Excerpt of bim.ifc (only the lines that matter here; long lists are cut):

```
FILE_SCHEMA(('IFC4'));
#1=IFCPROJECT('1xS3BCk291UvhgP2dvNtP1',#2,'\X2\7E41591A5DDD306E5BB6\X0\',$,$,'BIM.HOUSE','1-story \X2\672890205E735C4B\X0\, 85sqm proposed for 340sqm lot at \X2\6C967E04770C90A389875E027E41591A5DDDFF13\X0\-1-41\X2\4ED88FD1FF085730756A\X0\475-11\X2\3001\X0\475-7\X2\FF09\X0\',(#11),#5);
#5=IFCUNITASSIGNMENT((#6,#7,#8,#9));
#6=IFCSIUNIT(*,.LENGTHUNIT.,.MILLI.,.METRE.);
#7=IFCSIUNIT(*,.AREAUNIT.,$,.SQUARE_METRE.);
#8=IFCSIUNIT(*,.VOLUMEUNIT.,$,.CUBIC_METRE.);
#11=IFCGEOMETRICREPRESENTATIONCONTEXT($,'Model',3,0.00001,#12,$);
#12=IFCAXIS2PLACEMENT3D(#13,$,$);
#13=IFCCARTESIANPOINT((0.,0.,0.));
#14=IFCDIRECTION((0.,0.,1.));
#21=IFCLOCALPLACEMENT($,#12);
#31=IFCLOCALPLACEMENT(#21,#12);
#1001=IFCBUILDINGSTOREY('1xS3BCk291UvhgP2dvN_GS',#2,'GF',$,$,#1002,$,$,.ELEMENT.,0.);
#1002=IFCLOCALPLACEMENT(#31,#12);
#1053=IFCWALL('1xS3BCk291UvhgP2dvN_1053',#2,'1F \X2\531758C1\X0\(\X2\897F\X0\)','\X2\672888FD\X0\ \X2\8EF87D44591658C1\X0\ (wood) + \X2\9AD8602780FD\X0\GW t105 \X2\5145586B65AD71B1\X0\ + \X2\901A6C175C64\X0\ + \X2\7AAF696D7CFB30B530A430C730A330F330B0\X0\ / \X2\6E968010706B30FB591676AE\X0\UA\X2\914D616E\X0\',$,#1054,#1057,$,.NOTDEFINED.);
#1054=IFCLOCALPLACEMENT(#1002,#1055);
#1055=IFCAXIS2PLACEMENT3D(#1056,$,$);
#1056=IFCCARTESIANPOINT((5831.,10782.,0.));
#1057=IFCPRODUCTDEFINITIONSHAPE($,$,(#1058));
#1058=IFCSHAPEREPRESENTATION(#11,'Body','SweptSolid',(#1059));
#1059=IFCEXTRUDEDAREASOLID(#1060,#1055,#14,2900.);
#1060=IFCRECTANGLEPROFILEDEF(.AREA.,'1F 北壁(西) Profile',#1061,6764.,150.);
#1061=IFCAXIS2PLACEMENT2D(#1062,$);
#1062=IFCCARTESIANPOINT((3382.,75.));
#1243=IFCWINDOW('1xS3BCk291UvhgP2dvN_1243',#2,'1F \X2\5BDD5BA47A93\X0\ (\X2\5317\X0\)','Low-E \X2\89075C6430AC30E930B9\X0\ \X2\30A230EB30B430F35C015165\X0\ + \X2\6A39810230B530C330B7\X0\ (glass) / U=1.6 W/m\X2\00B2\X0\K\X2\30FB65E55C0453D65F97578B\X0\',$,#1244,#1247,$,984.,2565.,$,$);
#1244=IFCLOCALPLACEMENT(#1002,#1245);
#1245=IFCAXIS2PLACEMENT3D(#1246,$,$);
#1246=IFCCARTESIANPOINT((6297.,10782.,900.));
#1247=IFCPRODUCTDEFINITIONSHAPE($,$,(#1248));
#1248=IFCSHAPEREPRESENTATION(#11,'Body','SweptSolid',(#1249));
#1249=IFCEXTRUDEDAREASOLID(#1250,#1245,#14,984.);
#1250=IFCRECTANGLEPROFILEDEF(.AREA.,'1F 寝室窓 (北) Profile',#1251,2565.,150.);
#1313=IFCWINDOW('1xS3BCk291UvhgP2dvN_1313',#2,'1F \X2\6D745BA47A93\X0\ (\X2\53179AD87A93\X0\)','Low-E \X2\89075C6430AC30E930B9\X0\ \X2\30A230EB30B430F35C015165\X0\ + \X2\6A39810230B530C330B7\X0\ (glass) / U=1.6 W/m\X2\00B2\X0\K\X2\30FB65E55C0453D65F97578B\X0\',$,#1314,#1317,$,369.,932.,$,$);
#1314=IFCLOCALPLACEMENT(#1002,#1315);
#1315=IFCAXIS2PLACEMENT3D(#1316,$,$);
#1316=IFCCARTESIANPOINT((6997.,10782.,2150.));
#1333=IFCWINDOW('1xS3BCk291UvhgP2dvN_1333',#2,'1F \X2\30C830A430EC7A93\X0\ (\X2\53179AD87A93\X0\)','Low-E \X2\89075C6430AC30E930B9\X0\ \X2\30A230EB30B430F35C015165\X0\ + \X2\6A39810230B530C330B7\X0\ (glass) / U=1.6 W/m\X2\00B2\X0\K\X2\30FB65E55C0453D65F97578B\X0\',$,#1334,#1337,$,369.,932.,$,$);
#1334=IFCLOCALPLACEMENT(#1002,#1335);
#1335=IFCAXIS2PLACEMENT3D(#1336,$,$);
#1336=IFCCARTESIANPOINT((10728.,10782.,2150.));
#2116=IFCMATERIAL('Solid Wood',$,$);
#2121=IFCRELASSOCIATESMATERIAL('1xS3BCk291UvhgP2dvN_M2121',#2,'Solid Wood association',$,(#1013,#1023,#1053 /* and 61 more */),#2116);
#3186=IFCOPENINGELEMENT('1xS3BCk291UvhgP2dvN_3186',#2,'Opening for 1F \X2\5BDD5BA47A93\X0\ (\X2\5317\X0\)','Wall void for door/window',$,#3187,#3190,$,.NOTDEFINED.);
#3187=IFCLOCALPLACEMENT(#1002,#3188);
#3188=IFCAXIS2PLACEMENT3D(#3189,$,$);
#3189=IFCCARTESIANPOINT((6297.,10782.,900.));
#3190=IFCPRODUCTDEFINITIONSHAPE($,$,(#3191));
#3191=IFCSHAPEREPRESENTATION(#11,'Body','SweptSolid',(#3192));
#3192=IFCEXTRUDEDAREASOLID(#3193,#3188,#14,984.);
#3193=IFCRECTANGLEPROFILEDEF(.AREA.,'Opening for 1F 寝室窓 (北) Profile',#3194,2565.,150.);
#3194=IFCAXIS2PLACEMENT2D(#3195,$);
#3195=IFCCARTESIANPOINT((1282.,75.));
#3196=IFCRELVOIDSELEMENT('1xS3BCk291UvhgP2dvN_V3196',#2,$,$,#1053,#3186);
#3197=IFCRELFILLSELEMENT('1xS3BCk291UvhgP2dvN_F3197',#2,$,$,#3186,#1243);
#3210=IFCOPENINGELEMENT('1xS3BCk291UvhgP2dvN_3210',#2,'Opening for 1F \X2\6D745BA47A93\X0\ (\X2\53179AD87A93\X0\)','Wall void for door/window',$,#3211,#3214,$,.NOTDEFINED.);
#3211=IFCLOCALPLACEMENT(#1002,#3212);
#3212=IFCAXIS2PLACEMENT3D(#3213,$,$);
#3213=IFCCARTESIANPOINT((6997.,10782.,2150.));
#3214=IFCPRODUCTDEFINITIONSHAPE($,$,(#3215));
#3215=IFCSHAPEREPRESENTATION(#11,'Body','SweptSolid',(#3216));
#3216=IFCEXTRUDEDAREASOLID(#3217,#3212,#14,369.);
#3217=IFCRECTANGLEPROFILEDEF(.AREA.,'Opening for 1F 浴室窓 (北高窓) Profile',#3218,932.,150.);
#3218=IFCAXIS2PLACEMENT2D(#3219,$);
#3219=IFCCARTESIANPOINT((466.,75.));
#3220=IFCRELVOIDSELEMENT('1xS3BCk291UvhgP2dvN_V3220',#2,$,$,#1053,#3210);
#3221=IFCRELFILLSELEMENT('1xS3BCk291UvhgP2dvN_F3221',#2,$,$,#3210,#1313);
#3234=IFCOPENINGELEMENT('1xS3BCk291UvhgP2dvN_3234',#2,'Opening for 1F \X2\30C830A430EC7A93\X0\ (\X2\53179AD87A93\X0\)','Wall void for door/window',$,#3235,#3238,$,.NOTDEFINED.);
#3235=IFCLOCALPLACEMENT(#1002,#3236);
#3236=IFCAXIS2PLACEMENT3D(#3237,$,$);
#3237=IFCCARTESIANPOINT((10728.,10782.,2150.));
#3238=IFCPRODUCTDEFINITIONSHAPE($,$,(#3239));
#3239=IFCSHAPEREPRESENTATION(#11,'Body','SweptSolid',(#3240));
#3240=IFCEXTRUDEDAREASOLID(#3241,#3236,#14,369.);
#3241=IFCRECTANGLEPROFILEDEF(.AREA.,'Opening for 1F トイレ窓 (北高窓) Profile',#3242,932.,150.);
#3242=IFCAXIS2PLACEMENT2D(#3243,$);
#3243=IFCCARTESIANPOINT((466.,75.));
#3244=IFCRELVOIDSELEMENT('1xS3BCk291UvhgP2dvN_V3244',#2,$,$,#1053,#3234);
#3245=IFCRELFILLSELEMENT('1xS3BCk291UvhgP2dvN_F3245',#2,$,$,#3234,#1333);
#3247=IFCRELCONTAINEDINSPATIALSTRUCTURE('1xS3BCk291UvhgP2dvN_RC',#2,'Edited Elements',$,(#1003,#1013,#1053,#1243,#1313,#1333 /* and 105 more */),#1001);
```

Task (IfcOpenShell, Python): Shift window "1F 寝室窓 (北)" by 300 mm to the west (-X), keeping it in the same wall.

```python
import ifcopenshell
import ifcopenshell.api.geometry
import ifcopenshell.util.placement
import ifcopenshell.util.unit

model = ifcopenshell.open("bim.ifc")
unit_scale = ifcopenshell.util.unit.calculate_unit_scale(model)

window = model.by_guid("1xS3BCk291UvhgP2dvN_1243")
opening = window.FillsVoids[0].RelatingOpeningElement
wall = opening.VoidsElements[0].RelatingBuildingElement

wall_matrix = ifcopenshell.util.placement.get_local_placement(wall.ObjectPlacement)
shift = wall_matrix[:3, 0] * -0.3 / unit_scale
before = ifcopenshell.util.placement.get_local_placement(window.ObjectPlacement)[:3, 3].copy()

# The window is not placed relative to its opening, so move both.
for product in (opening, window):
    matrix = ifcopenshell.util.placement.get_local_placement(product.ObjectPlacement)
    matrix[:3, 3] += shift
    ifcopenshell.api.geometry.edit_object_placement(model, product=product, matrix=matrix, is_si=False)

after = ifcopenshell.util.placement.get_local_placement(window.ObjectPlacement)[:3, 3]
print("window moved by", (after - before).round(3) + 0.0)

model.write("bim_edited.ifc")
```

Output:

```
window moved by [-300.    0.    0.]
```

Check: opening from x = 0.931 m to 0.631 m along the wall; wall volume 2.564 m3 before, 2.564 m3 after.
